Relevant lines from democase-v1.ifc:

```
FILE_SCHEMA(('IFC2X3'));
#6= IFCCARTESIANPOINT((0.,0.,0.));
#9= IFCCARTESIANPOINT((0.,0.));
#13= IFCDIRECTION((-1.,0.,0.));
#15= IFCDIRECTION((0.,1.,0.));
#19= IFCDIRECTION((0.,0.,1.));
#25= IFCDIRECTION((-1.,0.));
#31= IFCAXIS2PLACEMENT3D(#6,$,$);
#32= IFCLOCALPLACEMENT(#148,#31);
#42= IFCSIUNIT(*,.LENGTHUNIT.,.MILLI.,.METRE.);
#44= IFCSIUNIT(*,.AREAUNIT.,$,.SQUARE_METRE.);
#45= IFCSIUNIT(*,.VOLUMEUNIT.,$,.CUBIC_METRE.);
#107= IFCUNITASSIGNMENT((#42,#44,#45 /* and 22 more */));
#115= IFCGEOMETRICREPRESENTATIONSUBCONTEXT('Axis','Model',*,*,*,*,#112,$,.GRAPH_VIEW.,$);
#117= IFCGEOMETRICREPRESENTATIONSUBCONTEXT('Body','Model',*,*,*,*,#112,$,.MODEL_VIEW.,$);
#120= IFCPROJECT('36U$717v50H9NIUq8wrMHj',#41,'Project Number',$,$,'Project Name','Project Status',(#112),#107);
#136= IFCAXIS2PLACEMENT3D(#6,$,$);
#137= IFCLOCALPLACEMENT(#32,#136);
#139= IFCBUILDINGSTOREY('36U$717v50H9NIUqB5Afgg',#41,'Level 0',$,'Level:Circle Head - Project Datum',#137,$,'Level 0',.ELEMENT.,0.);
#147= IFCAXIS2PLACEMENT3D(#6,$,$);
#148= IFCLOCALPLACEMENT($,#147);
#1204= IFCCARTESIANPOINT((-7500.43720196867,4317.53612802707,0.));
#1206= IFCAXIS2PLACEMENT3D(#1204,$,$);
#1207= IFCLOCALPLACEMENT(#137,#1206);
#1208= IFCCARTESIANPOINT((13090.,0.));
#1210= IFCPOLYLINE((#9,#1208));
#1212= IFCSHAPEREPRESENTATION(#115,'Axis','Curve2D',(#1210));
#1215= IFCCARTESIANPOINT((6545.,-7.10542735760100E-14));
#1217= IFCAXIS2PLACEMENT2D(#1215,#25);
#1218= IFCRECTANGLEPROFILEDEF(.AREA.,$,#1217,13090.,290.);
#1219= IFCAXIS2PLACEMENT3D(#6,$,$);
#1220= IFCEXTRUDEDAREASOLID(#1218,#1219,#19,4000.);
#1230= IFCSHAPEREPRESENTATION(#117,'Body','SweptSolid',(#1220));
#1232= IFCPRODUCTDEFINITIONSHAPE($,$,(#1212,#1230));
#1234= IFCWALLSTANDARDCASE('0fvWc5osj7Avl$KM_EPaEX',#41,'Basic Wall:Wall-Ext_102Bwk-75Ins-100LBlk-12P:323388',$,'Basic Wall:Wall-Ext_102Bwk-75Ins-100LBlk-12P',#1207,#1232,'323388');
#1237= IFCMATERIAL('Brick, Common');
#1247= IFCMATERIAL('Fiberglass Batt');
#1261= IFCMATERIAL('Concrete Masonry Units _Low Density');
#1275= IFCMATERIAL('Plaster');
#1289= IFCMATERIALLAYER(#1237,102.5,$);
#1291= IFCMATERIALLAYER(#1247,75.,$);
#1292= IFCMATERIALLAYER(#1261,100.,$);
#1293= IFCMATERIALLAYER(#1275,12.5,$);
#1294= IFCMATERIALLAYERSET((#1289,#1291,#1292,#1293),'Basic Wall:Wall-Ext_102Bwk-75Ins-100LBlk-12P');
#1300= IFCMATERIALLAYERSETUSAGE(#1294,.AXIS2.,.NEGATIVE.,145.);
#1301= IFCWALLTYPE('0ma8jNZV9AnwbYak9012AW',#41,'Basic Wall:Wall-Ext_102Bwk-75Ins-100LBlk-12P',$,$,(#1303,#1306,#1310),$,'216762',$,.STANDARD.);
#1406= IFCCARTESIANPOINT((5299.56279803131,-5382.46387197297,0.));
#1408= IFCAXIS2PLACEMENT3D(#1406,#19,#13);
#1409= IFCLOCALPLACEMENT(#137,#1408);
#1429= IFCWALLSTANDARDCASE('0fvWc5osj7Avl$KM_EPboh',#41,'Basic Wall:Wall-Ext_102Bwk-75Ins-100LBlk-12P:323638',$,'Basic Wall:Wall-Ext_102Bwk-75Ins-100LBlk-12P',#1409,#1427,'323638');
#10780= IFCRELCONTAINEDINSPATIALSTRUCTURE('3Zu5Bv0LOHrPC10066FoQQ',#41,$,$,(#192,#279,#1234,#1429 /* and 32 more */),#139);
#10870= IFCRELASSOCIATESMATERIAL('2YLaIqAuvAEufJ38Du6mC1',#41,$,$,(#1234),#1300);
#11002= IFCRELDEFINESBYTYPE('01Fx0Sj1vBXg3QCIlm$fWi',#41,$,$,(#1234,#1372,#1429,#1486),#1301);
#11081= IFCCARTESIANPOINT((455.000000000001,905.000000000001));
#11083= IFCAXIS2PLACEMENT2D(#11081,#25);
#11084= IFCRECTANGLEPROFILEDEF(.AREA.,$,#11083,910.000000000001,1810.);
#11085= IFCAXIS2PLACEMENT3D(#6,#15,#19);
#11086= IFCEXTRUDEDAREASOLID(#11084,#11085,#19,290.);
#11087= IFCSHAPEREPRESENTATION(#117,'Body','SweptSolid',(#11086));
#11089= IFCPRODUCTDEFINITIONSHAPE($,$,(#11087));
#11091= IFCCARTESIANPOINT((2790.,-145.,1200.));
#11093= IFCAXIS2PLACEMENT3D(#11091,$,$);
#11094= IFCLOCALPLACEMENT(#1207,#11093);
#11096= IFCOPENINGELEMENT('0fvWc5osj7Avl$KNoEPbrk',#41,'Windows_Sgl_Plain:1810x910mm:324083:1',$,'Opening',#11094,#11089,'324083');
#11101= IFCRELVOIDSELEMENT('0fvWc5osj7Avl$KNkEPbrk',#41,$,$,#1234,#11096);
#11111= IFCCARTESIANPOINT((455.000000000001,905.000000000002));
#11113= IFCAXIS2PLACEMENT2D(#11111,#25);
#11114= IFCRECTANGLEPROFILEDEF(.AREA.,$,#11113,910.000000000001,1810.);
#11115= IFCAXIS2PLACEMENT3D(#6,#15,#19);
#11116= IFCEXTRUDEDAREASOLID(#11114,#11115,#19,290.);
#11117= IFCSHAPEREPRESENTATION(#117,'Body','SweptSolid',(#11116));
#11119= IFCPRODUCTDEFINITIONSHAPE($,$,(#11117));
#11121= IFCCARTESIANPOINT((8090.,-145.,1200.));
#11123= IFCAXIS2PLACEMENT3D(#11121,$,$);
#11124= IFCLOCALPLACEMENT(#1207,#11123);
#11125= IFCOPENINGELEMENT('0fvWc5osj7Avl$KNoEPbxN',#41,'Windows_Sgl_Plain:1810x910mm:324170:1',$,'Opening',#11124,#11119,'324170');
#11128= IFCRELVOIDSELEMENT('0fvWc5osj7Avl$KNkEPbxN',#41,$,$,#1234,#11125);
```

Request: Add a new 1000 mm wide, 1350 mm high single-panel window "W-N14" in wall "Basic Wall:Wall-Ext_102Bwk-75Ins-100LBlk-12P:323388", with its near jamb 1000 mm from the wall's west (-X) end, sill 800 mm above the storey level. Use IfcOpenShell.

```python
import numpy as np
import ifcopenshell
import ifcopenshell.api.feature
import ifcopenshell.api.geometry
import ifcopenshell.api.root
import ifcopenshell.api.spatial
import ifcopenshell.api.type
import ifcopenshell.geom
import ifcopenshell.util.element
import ifcopenshell.util.placement
import ifcopenshell.util.representation
import ifcopenshell.util.shape
import ifcopenshell.util.unit

model = ifcopenshell.open("democase-v1.ifc")
unit_scale = ifcopenshell.util.unit.calculate_unit_scale(model)
settings = ifcopenshell.geom.settings()


def volume(element):
    """Net volume in cubic metres, openings subtracted."""
    shape = ifcopenshell.geom.create_shape(settings, element)
    return ifcopenshell.util.shape.get_volume(shape.geometry)


wall = model.by_id(1234)
storey = ifcopenshell.util.element.get_container(wall, ifc_class="IfcBuildingStorey")
context = ifcopenshell.util.representation.get_context(model, "Model", "Body", "MODEL_VIEW")
before = volume(wall)

width, height, from_end, sill = 1, 1.35, 1, 0.8  # metres

# The wall runs along its own X axis, and the end named is its -X end.
wall_shape = ifcopenshell.geom.create_shape(settings, wall)
x, y, z = ifcopenshell.util.shape.get_vertices(wall_shape.geometry).T
start = x.min() + from_end
face, thickness = float(y.min()), float(y.max() - y.min())
wall_matrix = ifcopenshell.util.placement.get_local_placement(wall.ObjectPlacement)
level = ifcopenshell.util.placement.get_local_placement(storey.ObjectPlacement)[2, 3]


def in_wall(x, y):
    """Placement at x, y metres in the wall's axes, at sill height."""
    matrix = wall_matrix.copy()
    matrix[:, 3] = wall_matrix @ np.array([x / unit_scale, y / unit_scale, 0.0, 1.0])
    matrix[2, 3] = level + sill / unit_scale
    return matrix


# Opening: a box that overshoots both wall faces by 50 mm.
opening = ifcopenshell.api.root.create_entity(model, ifc_class="IfcOpeningElement")
box = ifcopenshell.api.geometry.add_wall_representation(
    model, context=context, length=width, height=height, thickness=thickness + 0.1
)
ifcopenshell.api.geometry.assign_representation(model, product=opening, representation=box)
ifcopenshell.api.geometry.edit_object_placement(model, product=opening, matrix=in_wall(start, face - 0.05), is_si=False)
ifcopenshell.api.feature.add_feature(model, feature=opening, element=wall)

window = ifcopenshell.api.root.create_entity(model, ifc_class="IfcWindow", name="W-N14")
window.OverallWidth, window.OverallHeight = width / unit_scale, height / unit_scale
body = ifcopenshell.api.geometry.add_window_representation(
    model,
    context=context,
    overall_width=window.OverallWidth,
    overall_height=window.OverallHeight,
    partition_type="SINGLE_PANEL",
)
ifcopenshell.api.geometry.assign_representation(model, product=window, representation=body)
ifcopenshell.api.spatial.assign_container(model, products=[window], relating_structure=storey)
fills = ifcopenshell.api.feature.add_filling(model, opening=opening, element=window)
fills.OwnerHistory = window.OwnerHistory  # required in IFC2X3

# IFC2X3 keeps the operation on the window style.
style = ifcopenshell.api.root.create_entity(model, ifc_class="IfcWindowStyle", name="W-N14")
style.OperationType, style.ConstructionType = "SINGLE_PANEL", "NOTDEFINED"
style.ParameterTakesPrecedence = style.Sizeable = False
ifcopenshell.api.type.assign_type(model, related_objects=[window], relating_type=style)

# Centre the window in the wall's thickness.
ifcopenshell.api.geometry.edit_object_placement(model, product=window, matrix=in_wall(start, face), is_si=False)
window_shape = ifcopenshell.geom.create_shape(settings, window)
depth = ifcopenshell.util.shape.get_vertices(window_shape.geometry)[:, 1]
offset = face + thickness / 2 - (depth.min() + depth.max()) / 2
ifcopenshell.api.geometry.edit_object_placement(model, product=window, matrix=in_wall(start, offset), is_si=False)

after = volume(wall)

print(f"wall volume {before:.3f} -> {after:.3f} m3")

model.write("democase-v1_v2.ifc")
```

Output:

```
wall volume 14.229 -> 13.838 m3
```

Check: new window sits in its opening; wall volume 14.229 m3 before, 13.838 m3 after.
